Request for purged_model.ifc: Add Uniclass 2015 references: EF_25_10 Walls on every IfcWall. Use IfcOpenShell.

First a look at what the model holds.

```python
import ifcopenshell

model = ifcopenshell.open("purged_model.ifc")
print(model.schema)
print("classifications:", [c.Name for c in model.by_type("IfcClassification")])
for ifc_class in ("IfcDoor", "IfcRoof", "IfcStair", "IfcWall", "IfcWindow"):
    print(ifc_class, len(model.by_type(ifc_class)))
```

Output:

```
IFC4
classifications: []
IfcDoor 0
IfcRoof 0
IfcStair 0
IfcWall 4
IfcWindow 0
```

```python
import ifcopenshell
import ifcopenshell.api.classification

model = ifcopenshell.open("purged_model.ifc")

system = ifcopenshell.api.classification.add_classification(model, classification="Uniclass 2015")

codes = {
    "IfcWall": ("EF_25_10", "Walls"),
}
for ifc_class, (code, name) in codes.items():
    products = model.by_type(ifc_class)
    ifcopenshell.api.classification.add_reference(
        model, products=products, classification=system, identification=code, name=name
    )
    print(code, len(products))

model.write("purged_model-out.ifc")
```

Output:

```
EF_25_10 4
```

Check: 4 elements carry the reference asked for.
